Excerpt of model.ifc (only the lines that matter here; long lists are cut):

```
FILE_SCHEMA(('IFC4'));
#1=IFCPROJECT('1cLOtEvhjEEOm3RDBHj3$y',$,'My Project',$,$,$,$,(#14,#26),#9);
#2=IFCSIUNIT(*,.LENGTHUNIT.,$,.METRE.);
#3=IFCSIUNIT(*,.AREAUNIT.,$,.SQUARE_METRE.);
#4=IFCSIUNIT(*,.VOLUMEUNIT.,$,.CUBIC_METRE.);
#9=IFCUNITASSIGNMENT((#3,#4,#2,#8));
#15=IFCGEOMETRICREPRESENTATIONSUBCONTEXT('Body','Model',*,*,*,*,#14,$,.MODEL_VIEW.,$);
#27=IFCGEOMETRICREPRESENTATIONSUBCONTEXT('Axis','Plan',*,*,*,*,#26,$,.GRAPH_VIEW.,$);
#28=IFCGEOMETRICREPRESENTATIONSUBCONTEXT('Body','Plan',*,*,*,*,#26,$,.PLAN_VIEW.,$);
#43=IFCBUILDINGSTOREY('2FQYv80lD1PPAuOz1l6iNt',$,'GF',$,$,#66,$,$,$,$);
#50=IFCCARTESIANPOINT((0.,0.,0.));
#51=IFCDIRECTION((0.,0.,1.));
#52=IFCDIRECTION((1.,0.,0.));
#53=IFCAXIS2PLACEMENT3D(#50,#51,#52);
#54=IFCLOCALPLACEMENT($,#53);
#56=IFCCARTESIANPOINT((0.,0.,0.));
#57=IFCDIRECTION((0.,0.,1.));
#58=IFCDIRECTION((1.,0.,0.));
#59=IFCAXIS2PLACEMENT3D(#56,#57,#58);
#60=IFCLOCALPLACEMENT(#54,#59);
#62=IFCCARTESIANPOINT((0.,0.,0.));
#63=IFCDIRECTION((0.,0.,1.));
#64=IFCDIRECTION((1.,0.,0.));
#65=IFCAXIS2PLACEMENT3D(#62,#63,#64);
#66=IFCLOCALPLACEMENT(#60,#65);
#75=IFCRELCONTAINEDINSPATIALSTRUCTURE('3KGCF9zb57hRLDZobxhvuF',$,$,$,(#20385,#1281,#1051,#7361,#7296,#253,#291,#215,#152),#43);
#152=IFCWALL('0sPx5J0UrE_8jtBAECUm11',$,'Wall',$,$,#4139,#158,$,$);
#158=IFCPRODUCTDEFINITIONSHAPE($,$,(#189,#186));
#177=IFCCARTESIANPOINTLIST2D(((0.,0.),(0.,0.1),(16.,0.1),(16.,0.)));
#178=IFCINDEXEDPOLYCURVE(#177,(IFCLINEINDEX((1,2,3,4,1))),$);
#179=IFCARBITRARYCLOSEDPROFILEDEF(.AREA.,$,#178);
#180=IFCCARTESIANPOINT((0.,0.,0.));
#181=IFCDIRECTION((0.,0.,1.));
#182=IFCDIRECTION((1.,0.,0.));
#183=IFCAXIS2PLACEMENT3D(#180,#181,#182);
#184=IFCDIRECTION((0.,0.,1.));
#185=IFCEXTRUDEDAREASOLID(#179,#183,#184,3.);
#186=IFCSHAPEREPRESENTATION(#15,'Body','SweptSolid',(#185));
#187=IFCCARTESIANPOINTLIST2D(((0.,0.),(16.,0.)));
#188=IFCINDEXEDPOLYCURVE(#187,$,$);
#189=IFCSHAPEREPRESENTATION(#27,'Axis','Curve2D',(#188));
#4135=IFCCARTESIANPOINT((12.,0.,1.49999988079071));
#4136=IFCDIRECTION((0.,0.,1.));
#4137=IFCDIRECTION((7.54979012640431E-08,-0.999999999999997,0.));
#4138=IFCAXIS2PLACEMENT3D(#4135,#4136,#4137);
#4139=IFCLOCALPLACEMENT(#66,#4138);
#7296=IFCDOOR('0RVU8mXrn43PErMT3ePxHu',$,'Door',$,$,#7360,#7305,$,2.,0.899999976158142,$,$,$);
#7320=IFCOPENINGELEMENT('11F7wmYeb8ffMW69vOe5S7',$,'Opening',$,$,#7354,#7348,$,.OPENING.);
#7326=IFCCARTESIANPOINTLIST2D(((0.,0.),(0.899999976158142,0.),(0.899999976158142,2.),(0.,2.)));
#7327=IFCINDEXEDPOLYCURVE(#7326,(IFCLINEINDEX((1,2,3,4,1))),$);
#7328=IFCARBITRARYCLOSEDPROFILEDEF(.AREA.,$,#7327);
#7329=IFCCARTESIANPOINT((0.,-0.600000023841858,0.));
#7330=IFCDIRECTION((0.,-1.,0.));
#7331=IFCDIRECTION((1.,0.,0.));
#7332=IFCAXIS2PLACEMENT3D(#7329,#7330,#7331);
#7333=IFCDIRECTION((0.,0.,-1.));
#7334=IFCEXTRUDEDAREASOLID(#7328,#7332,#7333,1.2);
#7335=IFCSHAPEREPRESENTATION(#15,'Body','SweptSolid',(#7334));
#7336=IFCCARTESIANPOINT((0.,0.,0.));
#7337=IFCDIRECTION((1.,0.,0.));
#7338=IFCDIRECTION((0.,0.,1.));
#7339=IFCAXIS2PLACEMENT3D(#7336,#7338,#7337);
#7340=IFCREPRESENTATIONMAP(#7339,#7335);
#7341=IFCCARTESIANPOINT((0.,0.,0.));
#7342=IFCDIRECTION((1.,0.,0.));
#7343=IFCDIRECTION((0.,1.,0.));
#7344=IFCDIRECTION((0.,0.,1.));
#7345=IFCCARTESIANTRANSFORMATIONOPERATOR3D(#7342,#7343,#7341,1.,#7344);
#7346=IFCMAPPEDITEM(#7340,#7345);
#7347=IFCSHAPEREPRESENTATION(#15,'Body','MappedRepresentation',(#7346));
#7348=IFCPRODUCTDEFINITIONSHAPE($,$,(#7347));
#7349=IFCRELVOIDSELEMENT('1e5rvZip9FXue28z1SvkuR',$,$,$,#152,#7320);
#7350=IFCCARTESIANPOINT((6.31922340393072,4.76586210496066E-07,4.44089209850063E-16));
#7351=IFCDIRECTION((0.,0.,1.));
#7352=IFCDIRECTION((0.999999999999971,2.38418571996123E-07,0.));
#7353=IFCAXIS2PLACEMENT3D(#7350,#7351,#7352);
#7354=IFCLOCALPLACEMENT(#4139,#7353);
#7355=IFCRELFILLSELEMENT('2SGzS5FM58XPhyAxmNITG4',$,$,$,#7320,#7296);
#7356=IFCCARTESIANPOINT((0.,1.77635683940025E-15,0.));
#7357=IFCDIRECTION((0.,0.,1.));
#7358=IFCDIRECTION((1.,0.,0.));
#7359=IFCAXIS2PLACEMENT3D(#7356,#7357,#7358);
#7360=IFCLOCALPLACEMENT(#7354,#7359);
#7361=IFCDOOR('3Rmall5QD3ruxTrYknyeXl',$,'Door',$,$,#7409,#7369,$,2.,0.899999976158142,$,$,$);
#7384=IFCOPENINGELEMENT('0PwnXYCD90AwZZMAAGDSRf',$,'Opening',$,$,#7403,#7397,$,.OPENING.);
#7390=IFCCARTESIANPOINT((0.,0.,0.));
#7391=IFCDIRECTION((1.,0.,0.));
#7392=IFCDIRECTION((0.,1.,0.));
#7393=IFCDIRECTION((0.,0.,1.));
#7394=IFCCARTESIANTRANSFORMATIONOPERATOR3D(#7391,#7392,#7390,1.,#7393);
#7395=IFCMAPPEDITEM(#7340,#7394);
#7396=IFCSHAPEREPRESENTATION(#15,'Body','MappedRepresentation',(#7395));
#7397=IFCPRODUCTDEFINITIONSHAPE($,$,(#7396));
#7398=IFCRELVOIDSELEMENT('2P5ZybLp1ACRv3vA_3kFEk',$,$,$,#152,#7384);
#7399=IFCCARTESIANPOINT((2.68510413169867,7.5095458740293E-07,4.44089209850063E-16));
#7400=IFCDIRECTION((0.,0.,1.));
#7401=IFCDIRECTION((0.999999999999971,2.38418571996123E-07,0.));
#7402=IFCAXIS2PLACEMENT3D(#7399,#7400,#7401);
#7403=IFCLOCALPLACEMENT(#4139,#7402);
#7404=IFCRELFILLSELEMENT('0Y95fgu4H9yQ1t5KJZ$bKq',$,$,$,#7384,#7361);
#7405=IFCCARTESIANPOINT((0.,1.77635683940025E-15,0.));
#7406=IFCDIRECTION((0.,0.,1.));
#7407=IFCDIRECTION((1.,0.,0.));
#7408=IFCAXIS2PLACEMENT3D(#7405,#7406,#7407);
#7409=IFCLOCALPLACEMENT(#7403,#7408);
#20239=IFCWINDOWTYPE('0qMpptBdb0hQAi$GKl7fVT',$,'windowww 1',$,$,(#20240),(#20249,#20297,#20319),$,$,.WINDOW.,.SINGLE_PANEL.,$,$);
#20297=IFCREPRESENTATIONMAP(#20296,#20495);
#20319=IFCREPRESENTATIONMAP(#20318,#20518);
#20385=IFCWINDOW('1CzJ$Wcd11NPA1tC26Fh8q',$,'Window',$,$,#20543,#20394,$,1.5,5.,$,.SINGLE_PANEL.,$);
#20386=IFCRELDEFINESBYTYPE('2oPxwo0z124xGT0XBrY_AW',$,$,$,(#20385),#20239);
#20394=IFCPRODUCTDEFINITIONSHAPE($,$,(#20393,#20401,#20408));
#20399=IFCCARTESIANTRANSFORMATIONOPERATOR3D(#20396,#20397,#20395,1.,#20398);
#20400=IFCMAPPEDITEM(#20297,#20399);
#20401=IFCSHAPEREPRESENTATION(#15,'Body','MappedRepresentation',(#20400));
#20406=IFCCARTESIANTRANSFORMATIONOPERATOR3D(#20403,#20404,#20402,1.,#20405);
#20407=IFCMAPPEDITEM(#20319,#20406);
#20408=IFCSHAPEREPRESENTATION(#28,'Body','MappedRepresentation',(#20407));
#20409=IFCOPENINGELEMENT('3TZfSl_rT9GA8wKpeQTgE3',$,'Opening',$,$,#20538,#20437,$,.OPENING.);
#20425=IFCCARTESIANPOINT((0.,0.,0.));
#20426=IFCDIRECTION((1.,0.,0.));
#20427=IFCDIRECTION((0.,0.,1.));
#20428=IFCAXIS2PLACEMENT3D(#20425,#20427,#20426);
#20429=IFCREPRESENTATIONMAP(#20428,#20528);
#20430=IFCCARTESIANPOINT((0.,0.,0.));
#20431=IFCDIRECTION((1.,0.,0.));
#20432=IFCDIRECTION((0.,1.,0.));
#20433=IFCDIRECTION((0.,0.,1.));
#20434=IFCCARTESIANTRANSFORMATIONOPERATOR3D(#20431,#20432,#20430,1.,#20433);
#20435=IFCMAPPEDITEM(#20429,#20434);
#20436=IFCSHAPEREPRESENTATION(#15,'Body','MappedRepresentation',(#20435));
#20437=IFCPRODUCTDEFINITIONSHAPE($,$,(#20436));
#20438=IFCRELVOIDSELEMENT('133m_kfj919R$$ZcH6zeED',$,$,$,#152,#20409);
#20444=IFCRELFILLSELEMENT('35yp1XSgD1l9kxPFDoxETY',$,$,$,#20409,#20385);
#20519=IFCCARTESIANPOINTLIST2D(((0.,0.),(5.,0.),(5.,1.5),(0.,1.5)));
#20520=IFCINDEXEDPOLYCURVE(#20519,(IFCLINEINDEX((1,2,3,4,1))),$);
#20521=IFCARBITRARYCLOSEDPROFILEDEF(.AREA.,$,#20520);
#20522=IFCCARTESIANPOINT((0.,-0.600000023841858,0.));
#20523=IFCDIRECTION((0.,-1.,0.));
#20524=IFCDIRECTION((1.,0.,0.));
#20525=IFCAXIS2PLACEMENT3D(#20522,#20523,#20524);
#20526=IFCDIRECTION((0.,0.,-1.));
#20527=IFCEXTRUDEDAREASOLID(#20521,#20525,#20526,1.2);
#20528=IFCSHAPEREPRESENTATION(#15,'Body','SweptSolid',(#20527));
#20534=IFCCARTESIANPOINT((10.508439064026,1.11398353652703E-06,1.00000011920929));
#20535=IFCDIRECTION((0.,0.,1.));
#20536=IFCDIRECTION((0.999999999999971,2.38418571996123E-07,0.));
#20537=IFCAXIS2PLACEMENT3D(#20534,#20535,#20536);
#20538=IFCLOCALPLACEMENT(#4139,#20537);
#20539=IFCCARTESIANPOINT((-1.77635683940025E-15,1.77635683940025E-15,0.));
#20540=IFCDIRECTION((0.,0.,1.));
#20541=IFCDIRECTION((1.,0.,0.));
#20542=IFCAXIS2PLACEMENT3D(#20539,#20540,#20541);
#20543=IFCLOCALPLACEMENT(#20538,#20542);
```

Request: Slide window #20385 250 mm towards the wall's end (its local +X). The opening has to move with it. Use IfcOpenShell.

```python
import ifcopenshell
import ifcopenshell.api.geometry
import ifcopenshell.util.placement
import ifcopenshell.util.unit

model = ifcopenshell.open("model.ifc")
unit_scale = ifcopenshell.util.unit.calculate_unit_scale(model)

window = model.by_guid("1CzJ$Wcd11NPA1tC26Fh8q")
opening = window.FillsVoids[0].RelatingOpeningElement
wall = opening.VoidsElements[0].RelatingBuildingElement

wall_matrix = ifcopenshell.util.placement.get_local_placement(wall.ObjectPlacement)
shift = wall_matrix[:3, 0] * 0.25 / unit_scale
before = ifcopenshell.util.placement.get_local_placement(window.ObjectPlacement)[:3, 3].copy()

# The window is placed relative to its opening, so it follows when the opening moves.
matrix = ifcopenshell.util.placement.get_local_placement(opening.ObjectPlacement)
matrix[:3, 3] += shift
ifcopenshell.api.geometry.edit_object_placement(
    model, product=opening, matrix=matrix, is_si=False, should_transform_children=True
)

after = ifcopenshell.util.placement.get_local_placement(window.ObjectPlacement)[:3, 3]
print("window moved by", (after - before).round(3) + 0.0)

model.write("model_updated.ifc")
```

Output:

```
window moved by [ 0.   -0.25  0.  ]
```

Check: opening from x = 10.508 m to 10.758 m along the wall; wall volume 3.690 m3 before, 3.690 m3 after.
